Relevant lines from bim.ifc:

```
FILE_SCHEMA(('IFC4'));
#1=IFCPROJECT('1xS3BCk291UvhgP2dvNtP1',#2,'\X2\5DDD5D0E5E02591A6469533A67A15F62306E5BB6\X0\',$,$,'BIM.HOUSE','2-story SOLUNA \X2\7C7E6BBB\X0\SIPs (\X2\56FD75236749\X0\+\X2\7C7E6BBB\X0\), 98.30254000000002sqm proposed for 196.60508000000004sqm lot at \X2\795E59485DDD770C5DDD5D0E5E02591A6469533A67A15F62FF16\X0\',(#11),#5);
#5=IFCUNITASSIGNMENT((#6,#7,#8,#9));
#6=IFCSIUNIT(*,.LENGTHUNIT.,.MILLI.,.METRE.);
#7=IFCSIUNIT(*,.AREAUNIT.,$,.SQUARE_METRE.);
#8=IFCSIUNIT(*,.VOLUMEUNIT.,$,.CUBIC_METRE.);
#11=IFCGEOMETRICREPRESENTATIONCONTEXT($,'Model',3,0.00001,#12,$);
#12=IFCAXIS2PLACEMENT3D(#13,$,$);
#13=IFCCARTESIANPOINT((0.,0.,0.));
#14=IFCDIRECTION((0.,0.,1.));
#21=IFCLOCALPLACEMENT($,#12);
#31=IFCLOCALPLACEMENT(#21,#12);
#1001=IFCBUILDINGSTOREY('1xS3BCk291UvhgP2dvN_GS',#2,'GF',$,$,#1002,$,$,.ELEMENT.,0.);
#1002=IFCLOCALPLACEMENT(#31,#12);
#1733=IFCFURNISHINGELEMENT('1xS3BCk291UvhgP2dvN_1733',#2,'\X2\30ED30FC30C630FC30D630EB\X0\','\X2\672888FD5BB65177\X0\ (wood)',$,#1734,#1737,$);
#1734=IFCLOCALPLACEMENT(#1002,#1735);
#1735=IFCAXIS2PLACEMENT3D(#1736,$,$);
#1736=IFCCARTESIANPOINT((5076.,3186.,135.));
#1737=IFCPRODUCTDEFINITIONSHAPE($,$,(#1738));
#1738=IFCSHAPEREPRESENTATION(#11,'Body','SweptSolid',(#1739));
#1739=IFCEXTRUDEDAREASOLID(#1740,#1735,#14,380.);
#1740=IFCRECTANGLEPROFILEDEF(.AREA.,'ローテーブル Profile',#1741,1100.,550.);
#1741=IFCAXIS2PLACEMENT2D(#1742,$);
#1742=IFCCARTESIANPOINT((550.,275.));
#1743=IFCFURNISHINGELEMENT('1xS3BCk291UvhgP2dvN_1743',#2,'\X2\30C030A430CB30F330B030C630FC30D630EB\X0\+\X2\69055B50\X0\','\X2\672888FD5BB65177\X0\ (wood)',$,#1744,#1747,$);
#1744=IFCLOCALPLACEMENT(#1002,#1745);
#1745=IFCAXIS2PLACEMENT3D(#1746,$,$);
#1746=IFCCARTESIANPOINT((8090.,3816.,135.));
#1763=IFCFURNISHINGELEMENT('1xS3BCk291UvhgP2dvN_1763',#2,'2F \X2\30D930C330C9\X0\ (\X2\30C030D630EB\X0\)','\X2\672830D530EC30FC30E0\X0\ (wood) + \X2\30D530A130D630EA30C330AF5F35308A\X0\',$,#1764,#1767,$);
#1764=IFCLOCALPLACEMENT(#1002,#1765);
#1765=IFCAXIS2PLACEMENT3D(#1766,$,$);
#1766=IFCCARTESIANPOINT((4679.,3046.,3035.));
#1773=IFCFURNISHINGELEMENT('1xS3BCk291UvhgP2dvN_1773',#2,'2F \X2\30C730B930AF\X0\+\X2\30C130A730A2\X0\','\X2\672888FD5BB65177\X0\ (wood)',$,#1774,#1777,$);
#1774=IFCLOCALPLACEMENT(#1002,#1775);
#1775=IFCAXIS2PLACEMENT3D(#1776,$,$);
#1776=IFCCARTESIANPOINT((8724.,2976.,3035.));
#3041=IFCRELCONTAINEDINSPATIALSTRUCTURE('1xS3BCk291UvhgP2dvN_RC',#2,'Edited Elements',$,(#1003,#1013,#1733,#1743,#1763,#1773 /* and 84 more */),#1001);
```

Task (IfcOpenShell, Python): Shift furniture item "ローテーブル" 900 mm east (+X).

```python
import ifcopenshell
import ifcopenshell.api.geometry
import ifcopenshell.util.placement

model = ifcopenshell.open("bim.ifc")

item = model.by_guid("1xS3BCk291UvhgP2dvN_1733")
matrix = ifcopenshell.util.placement.get_local_placement(item.ObjectPlacement)
matrix[0, 3] += 900.0
ifcopenshell.api.geometry.edit_object_placement(model, product=item, matrix=matrix, is_si=False)

print(ifcopenshell.util.placement.get_local_placement(item.ObjectPlacement).round(3) + 0.0)

model.write("bim_rev.ifc")
```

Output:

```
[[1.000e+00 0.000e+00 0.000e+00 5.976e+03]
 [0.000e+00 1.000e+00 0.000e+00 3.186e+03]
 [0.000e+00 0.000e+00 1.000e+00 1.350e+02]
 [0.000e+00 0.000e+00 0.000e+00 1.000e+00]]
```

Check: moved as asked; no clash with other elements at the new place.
